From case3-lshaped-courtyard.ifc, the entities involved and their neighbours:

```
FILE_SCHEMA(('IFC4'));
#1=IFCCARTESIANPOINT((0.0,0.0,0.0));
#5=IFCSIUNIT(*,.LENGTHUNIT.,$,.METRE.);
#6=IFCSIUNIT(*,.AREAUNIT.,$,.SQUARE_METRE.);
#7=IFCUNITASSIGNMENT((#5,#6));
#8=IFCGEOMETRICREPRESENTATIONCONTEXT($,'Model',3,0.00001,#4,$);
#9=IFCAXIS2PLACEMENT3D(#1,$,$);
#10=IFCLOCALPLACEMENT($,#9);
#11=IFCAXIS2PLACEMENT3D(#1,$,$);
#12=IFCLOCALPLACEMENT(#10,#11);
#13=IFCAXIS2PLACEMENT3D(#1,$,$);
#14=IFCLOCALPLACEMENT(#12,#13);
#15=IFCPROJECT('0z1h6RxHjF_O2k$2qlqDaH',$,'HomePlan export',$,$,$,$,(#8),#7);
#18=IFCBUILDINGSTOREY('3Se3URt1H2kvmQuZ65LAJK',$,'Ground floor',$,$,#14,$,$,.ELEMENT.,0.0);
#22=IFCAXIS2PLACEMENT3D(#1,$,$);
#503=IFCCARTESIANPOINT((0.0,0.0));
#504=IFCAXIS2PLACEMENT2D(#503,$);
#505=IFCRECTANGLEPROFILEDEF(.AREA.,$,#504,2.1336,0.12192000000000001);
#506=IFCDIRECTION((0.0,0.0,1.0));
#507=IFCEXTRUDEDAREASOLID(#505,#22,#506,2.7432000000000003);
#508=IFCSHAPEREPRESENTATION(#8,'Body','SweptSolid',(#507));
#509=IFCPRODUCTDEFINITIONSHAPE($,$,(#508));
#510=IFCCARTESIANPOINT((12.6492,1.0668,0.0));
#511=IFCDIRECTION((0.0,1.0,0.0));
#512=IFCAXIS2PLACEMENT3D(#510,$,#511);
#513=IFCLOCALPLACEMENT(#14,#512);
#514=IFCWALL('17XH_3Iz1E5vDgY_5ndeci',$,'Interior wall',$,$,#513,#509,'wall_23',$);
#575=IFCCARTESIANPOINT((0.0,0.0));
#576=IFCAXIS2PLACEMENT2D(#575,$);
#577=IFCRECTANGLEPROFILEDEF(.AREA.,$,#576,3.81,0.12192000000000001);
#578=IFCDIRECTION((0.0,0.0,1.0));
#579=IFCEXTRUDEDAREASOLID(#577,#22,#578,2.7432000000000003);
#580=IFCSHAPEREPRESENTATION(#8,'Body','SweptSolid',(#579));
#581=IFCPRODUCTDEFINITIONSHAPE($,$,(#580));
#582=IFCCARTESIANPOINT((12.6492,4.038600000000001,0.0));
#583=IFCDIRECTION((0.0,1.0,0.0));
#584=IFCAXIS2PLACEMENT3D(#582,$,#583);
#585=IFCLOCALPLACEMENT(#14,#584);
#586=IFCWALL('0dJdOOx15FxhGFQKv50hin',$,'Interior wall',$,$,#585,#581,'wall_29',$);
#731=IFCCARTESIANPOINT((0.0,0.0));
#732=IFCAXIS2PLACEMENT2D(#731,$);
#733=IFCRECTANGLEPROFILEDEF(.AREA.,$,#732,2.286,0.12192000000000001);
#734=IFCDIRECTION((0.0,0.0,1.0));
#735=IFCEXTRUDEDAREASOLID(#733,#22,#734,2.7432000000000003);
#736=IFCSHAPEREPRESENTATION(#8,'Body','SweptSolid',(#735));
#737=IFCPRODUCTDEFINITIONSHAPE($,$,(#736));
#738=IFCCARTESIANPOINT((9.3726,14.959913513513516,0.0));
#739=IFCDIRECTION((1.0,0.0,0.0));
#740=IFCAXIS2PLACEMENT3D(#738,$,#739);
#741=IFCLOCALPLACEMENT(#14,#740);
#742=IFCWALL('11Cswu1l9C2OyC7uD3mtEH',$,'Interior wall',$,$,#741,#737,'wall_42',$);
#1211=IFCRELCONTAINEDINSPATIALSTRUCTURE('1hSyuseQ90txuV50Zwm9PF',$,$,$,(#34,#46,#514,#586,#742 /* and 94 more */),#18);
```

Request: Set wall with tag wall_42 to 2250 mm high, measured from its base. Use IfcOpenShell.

```python
import ifcopenshell
import ifcopenshell.geom
import ifcopenshell.util.shape

model = ifcopenshell.open("case3-lshaped-courtyard.ifc")
settings = ifcopenshell.geom.settings()


def volume(element):
    """Net volume in cubic metres, openings subtracted."""
    shape = ifcopenshell.geom.create_shape(settings, element)
    return ifcopenshell.util.shape.get_volume(shape.geometry)


wall = model.by_guid("11Cswu1l9C2OyC7uD3mtEH")
before = volume(wall)

body = next(r for r in wall.Representation.Representations if r.RepresentationIdentifier == "Body")
solid = body.Items[0]
old_height = solid.Depth
solid.Depth = 2.25
after = volume(wall)

print(f"height {old_height:g} -> {solid.Depth:g}, volume {before:.3f} -> {after:.3f} m3")

model.write("case3-lshaped-courtyard-out.ifc")
```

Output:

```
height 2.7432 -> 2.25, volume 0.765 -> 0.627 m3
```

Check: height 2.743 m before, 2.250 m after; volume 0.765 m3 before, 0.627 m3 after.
